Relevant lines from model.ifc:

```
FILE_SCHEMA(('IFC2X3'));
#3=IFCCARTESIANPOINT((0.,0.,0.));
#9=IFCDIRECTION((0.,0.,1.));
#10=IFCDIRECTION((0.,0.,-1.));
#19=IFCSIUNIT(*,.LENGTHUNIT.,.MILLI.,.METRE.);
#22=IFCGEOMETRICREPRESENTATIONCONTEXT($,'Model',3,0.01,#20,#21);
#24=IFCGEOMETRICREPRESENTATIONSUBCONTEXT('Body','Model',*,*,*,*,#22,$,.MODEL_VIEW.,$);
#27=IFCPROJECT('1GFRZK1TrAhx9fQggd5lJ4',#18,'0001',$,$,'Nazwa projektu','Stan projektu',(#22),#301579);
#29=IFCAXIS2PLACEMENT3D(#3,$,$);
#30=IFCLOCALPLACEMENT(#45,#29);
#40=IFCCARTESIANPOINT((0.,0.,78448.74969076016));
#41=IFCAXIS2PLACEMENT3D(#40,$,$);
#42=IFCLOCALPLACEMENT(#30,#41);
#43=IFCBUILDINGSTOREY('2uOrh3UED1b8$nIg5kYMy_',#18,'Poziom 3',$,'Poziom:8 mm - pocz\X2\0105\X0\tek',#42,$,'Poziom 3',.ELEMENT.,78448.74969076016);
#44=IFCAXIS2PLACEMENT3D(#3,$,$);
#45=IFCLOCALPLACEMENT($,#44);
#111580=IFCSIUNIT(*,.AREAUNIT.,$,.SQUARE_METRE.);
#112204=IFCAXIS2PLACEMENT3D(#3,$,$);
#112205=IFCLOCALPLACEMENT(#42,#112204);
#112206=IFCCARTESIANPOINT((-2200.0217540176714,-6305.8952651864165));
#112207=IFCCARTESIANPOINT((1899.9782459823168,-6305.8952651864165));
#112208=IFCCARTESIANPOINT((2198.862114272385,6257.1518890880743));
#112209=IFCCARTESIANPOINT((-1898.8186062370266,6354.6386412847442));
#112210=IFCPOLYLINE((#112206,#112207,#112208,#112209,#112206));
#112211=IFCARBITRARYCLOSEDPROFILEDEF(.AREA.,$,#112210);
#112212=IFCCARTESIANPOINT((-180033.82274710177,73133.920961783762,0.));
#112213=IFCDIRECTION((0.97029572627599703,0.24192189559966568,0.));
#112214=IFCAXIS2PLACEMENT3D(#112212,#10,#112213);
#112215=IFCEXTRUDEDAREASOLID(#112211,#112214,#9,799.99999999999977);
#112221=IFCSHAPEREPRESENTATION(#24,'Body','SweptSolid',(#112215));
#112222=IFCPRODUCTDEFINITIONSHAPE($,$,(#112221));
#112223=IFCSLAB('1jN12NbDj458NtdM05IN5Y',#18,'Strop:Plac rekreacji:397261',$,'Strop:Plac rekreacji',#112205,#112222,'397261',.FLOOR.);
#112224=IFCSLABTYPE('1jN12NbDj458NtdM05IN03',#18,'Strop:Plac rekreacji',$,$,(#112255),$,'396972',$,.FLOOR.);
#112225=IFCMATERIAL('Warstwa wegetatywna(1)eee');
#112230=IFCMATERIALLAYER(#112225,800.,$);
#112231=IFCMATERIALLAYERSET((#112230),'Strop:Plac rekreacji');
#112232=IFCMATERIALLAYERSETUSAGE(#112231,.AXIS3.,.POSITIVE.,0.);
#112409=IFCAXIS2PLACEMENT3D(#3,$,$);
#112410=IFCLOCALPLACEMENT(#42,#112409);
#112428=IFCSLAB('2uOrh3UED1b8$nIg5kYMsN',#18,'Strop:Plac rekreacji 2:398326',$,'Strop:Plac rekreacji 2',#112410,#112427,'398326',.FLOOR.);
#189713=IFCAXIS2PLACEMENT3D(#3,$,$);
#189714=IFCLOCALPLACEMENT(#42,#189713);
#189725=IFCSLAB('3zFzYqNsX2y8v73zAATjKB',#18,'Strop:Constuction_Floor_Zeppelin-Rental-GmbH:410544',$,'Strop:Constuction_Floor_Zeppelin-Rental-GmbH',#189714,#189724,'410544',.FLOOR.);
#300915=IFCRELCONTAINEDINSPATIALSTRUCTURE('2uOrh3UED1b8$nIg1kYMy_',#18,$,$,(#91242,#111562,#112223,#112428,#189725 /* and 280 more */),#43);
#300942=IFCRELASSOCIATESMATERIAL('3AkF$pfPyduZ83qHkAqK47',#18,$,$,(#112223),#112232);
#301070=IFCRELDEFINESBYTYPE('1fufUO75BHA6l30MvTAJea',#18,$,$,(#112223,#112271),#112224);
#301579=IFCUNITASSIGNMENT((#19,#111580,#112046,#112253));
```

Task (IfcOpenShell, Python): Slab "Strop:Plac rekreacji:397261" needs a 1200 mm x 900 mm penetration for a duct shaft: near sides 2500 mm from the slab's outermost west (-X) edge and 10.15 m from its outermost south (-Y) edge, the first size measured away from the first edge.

```python
import numpy as np
import ifcopenshell
import ifcopenshell.api.feature
import ifcopenshell.api.geometry
import ifcopenshell.api.root
import ifcopenshell.geom
import ifcopenshell.util.placement
import ifcopenshell.util.representation
import ifcopenshell.util.shape
import ifcopenshell.util.unit

model = ifcopenshell.open("model.ifc")
unit_scale = ifcopenshell.util.unit.calculate_unit_scale(model)
settings = ifcopenshell.geom.settings()


def volume(element):
    """Net volume in cubic metres, openings subtracted."""
    shape = ifcopenshell.geom.create_shape(settings, element)
    return ifcopenshell.util.shape.get_volume(shape.geometry)


slab = model.by_guid("1jN12NbDj458NtdM05IN5Y")
before = volume(slab)

# Extent in the slab's own axes, in metres. The edges named are its -X and -Y sides.
slab_shape = ifcopenshell.geom.create_shape(settings, slab)
vertices = ifcopenshell.util.shape.get_vertices(slab_shape.geometry)
x_min, y_min, bottom = vertices.min(axis=0)
top = vertices[:, 2].max()

opening = ifcopenshell.api.root.create_entity(model, ifc_class="IfcOpeningElement", name="Duct shaft opening")
context = ifcopenshell.util.representation.get_context(model, "Model", "Body", "MODEL_VIEW")
width, depth = 1.2, 0.9
outline = [(0.0, 0.0), (width, 0.0), (width, depth), (0.0, depth), (0.0, 0.0)]
# Overshoot both faces by 50 mm so the cut is clean.
shape = ifcopenshell.api.geometry.add_slab_representation(
    model, context=context, depth=top - bottom + 0.1, polyline=outline
)
ifcopenshell.api.geometry.assign_representation(model, product=opening, representation=shape)

matrix = ifcopenshell.util.placement.get_local_placement(slab.ObjectPlacement)
matrix[:, 3] = matrix @ np.append(np.array([x_min + 2.5, y_min + 10.15, bottom - 0.05]) / unit_scale, 1.0)
ifcopenshell.api.geometry.edit_object_placement(model, product=opening, matrix=matrix, is_si=False)
ifcopenshell.api.feature.add_feature(model, feature=opening, element=slab)

after = volume(slab)

print(f"slab volume {before:.3f} -> {after:.3f} m3")

model.write("model_v2.ifc")
```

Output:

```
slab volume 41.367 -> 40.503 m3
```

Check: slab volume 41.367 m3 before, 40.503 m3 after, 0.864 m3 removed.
